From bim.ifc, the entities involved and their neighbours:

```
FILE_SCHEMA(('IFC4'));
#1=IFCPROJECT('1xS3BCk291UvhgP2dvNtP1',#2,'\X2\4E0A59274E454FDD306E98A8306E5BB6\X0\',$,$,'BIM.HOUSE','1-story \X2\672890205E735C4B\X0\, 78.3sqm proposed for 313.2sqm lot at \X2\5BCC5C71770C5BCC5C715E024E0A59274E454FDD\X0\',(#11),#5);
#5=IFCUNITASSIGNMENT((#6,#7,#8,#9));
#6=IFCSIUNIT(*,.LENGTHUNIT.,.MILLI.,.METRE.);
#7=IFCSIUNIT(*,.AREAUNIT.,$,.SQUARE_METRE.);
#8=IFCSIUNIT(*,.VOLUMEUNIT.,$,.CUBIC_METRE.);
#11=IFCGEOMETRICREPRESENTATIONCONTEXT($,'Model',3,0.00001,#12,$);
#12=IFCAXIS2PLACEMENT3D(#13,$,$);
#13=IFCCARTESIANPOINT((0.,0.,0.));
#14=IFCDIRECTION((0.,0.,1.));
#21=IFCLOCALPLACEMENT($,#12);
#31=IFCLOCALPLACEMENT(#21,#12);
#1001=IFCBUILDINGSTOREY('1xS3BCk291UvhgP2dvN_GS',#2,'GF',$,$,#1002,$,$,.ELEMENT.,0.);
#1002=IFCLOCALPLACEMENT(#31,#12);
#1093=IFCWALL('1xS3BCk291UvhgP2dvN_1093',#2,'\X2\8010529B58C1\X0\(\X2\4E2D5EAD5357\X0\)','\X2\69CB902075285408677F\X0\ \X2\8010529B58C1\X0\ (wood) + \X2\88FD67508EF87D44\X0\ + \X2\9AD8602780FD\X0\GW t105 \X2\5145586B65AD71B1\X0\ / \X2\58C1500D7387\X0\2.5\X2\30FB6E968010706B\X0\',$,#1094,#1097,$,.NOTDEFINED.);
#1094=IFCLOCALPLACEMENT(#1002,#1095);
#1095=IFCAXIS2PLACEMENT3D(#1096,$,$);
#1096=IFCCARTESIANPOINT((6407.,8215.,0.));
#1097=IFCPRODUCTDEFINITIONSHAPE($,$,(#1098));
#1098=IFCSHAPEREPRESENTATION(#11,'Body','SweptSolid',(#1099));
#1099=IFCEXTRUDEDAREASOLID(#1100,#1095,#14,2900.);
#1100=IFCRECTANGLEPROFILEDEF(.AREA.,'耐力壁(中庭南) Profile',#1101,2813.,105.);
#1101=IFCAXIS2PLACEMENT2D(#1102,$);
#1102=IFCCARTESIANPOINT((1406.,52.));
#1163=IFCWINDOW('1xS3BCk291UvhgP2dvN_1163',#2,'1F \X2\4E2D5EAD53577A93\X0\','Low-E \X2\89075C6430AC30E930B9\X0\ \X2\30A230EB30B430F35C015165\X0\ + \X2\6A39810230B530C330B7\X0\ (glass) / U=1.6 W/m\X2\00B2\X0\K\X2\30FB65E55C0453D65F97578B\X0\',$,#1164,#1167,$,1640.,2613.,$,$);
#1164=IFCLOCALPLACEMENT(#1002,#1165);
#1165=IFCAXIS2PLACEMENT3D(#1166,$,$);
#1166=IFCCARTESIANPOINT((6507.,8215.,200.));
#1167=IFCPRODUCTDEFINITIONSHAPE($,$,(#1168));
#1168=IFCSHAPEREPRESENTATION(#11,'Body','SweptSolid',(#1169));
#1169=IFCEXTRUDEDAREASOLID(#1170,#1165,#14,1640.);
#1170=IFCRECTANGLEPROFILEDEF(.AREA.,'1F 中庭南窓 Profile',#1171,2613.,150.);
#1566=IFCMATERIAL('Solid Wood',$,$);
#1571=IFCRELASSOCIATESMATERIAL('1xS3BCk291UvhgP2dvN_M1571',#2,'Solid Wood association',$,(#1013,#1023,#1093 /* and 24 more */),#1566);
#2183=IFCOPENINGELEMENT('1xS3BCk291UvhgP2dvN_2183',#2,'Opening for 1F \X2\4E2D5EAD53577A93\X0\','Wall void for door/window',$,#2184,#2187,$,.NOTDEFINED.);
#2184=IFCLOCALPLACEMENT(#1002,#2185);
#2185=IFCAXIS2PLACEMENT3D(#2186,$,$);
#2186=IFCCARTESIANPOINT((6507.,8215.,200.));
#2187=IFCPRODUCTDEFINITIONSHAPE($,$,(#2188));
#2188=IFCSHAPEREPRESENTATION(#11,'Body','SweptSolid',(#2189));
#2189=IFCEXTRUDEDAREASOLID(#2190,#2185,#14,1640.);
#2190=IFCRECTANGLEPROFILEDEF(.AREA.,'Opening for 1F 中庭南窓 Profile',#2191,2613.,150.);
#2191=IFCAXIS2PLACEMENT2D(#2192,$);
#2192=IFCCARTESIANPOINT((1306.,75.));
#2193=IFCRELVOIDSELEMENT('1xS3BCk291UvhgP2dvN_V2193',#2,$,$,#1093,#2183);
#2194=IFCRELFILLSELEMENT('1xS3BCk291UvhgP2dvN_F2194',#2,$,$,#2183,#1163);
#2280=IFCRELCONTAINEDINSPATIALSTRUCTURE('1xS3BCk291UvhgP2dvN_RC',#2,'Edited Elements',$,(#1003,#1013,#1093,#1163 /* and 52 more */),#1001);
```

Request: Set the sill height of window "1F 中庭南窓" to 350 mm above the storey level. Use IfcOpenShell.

```python
import numpy as np
import ifcopenshell
import ifcopenshell.api.geometry
import ifcopenshell.geom
import ifcopenshell.util.element
import ifcopenshell.util.placement
import ifcopenshell.util.shape
import ifcopenshell.util.unit

model = ifcopenshell.open("bim.ifc")
unit_scale = ifcopenshell.util.unit.calculate_unit_scale(model)

window = model.by_id(1163)
opening = window.FillsVoids[0].RelatingOpeningElement
storey = ifcopenshell.util.element.get_container(window, ifc_class="IfcBuildingStorey")
level = ifcopenshell.util.placement.get_local_placement(storey.ObjectPlacement)[2, 3]

# The opening's origin need not be at the sill, so measure its lowest point.
shape = ifcopenshell.geom.create_shape(ifcopenshell.geom.settings(), opening)
bottom = ifcopenshell.util.shape.get_shape_bottom_elevation(shape, shape.geometry) / unit_scale
dz = level + 0.35 / unit_scale - bottom

shift = np.array([0.0, 0.0, dz])
# The window is not placed relative to its opening, so move both.
for product in (opening, window):
    matrix = ifcopenshell.util.placement.get_local_placement(product.ObjectPlacement)
    matrix[:3, 3] += shift
    ifcopenshell.api.geometry.edit_object_placement(model, product=product, matrix=matrix, is_si=False)

print(f"moved by {dz * unit_scale:+.3f} m")

model.write("bim_v2.ifc")
```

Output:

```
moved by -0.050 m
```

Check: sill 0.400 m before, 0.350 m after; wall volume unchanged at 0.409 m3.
